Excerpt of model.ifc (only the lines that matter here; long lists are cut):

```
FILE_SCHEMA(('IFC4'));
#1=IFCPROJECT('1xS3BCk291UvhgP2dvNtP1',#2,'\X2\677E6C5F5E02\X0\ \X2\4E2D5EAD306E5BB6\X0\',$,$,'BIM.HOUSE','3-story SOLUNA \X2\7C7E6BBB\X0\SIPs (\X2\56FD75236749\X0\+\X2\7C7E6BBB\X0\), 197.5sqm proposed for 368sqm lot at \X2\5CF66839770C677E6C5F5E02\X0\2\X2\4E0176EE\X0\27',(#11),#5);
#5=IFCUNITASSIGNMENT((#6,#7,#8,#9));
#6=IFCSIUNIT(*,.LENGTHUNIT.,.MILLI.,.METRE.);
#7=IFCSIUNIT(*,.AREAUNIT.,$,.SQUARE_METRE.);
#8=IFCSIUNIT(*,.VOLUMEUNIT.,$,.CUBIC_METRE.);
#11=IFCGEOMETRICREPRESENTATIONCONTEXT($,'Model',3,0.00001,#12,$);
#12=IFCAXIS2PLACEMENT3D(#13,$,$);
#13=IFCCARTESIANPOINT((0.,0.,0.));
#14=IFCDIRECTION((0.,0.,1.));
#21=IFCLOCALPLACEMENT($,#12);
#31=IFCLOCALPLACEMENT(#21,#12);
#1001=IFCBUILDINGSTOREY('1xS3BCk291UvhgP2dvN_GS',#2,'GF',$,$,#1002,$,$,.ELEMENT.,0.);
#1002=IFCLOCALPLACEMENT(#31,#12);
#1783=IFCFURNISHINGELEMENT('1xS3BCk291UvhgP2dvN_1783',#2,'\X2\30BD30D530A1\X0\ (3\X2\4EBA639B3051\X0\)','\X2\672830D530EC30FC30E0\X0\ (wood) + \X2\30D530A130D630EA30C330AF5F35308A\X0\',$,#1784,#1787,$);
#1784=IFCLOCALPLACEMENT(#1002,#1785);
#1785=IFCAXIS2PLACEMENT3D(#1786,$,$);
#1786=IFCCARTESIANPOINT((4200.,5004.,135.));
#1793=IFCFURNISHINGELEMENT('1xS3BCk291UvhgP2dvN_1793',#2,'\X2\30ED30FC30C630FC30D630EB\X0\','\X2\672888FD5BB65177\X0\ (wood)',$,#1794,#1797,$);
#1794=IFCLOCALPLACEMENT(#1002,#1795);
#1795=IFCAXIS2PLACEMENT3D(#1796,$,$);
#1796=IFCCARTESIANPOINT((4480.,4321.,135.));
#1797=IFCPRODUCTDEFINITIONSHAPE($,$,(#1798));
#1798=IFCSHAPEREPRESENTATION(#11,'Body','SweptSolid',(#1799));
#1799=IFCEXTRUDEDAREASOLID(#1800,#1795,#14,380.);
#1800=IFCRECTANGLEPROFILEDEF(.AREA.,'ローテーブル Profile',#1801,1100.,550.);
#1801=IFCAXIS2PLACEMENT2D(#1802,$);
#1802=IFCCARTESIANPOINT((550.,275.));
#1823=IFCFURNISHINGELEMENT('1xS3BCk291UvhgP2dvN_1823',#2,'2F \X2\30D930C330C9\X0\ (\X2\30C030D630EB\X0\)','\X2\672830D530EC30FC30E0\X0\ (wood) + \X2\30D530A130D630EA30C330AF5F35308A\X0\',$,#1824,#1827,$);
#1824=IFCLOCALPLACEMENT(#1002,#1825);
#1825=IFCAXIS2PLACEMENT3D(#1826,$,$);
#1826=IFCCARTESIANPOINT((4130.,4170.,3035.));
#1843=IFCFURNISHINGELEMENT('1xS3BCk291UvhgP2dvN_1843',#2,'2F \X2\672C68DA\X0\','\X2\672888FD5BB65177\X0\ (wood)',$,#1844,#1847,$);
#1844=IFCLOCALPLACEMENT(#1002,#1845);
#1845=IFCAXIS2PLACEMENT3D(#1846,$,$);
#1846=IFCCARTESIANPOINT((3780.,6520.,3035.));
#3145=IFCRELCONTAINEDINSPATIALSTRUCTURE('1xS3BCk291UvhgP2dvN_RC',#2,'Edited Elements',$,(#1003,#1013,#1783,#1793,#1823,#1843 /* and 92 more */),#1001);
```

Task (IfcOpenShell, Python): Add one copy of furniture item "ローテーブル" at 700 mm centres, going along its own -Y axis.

```python
import ifcopenshell
import ifcopenshell.api.geometry
import ifcopenshell.api.root
import ifcopenshell.util.element
import ifcopenshell.util.placement
import ifcopenshell.util.unit

model = ifcopenshell.open("model.ifc")
unit_scale = ifcopenshell.util.unit.calculate_unit_scale(model)


def reuse_history(source, copy):
    """copy_class also copies each property set's owner history, people and application; keep the originals."""
    for rel in copy.IsDefinedBy:
        if rel.is_a("IfcRelDefinesByProperties") and (history := rel.RelatingPropertyDefinition.OwnerHistory):
            rel.RelatingPropertyDefinition.OwnerHistory = source.OwnerHistory
            ifcopenshell.util.element.remove_deep2(model, history)


source = model.by_guid("1xS3BCk291UvhgP2dvN_1793")
base = ifcopenshell.util.placement.get_local_placement(source.ObjectPlacement)
step = -base[:3, 1] * 0.7 / unit_scale

for i in range(1, 2):
    copy = ifcopenshell.api.root.copy_class(model, product=source)
    copy.Representation = ifcopenshell.util.element.copy_deep(
        model, source.Representation, exclude=["IfcGeometricRepresentationContext", "IfcRepresentationMap"]
    )
    reuse_history(source, copy)
    matrix = base.copy()
    matrix[:3, 3] += i * step
    print("added at", matrix[:3, 3].round(3) + 0.0)
    ifcopenshell.api.geometry.edit_object_placement(model, product=copy, matrix=matrix, is_si=False)

model.write("model_updated.ifc")
```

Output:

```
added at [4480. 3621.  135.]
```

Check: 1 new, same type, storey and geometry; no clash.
